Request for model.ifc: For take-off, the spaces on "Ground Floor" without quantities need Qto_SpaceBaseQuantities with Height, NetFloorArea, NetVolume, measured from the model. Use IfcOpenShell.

First a look at what the model holds.

```python
import ifcopenshell
import ifcopenshell.util.element
import ifcopenshell.util.unit

model = ifcopenshell.open("model.ifc")
print(model.schema)
for unit_type in ("LENGTHUNIT", "AREAUNIT", "VOLUMEUNIT"):
    print(unit_type, ifcopenshell.util.unit.calculate_unit_scale(model, unit_type))
storey = next(s for s in model.by_type("IfcBuildingStorey") if s.Name == "Ground Floor")
spaces = [e for e in ifcopenshell.util.element.get_decomposition(storey) if e.is_a("IfcSpace")]
for e in sorted(spaces, key=lambda e: e.id()):
    print(e.id(), e.is_a(), e.Name, list(ifcopenshell.util.element.get_psets(e, qtos_only=True)), sep=" | ")
```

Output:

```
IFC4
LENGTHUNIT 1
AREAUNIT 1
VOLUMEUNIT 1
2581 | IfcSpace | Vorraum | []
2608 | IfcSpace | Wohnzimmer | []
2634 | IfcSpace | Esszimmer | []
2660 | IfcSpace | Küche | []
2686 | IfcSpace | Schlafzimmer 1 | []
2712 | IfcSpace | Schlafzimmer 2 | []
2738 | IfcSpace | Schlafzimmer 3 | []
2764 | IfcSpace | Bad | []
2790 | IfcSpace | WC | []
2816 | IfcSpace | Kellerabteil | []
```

```python
import ifcopenshell
import ifcopenshell.api.pset
import ifcopenshell.geom
import ifcopenshell.util.element
import ifcopenshell.util.shape
import ifcopenshell.util.unit

model = ifcopenshell.open("model.ifc")
unit_scale = ifcopenshell.util.unit.calculate_unit_scale(model)
area_scale = ifcopenshell.util.unit.calculate_unit_scale(model, "AREAUNIT")
volume_scale = ifcopenshell.util.unit.calculate_unit_scale(model, "VOLUMEUNIT")
settings = ifcopenshell.geom.settings()

storey = next(s for s in model.by_type("IfcBuildingStorey") if s.Name == "Ground Floor")
spaces = [e for e in ifcopenshell.util.element.get_decomposition(storey) if e.is_a("IfcSpace")]

for e in sorted(spaces, key=lambda e: e.id()):
    if ifcopenshell.util.element.get_psets(e, qtos_only=True, should_inherit=False):
        continue
    # Geometry comes back in metres, in the element's own axes.
    shape = ifcopenshell.geom.create_shape(settings, e)
    values = {
        "Height": ifcopenshell.util.shape.get_z(shape.geometry) / unit_scale,
        "NetFloorArea": ifcopenshell.util.shape.get_footprint_area(shape.geometry) / area_scale,
        "NetVolume": ifcopenshell.util.shape.get_volume(shape.geometry) / volume_scale,
    }
    qto = ifcopenshell.api.pset.add_qto(model, product=e, name="Qto_SpaceBaseQuantities")
    ifcopenshell.api.pset.edit_qto(model, qto=qto, properties=values)
    print(e.id(), {k: round(v, 3) for k, v in values.items()})

model.write("model-out.ifc")
```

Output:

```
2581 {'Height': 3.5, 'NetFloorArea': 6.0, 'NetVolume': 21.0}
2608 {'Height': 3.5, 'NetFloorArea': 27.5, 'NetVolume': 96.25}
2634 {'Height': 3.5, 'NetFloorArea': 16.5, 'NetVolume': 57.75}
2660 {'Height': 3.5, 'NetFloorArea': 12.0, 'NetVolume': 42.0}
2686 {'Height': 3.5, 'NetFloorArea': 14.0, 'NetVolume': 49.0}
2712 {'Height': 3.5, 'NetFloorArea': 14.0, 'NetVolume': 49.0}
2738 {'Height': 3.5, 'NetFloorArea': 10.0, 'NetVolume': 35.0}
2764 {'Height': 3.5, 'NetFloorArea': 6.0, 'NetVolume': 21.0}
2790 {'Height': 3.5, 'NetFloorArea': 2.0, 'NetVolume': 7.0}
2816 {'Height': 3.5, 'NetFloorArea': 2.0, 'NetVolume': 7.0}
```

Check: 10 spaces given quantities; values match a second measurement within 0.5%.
